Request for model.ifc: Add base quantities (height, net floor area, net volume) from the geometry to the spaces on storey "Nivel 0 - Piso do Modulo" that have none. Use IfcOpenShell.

First a look at what the model holds.

```python
import ifcopenshell
import ifcopenshell.util.element
import ifcopenshell.util.unit

model = ifcopenshell.open("model.ifc")
print(model.schema)
for unit_type in ("LENGTHUNIT", "AREAUNIT", "VOLUMEUNIT"):
    print(unit_type, ifcopenshell.util.unit.calculate_unit_scale(model, unit_type))
storey = next(s for s in model.by_type("IfcBuildingStorey") if s.Name == "Nivel 0 - Piso do Modulo")
spaces = [e for e in ifcopenshell.util.element.get_decomposition(storey) if e.is_a("IfcSpace")]
for e in sorted(spaces, key=lambda e: e.id()):
    print(e.id(), e.is_a(), e.Name, list(ifcopenshell.util.element.get_psets(e, qtos_only=True)), sep=" | ")
```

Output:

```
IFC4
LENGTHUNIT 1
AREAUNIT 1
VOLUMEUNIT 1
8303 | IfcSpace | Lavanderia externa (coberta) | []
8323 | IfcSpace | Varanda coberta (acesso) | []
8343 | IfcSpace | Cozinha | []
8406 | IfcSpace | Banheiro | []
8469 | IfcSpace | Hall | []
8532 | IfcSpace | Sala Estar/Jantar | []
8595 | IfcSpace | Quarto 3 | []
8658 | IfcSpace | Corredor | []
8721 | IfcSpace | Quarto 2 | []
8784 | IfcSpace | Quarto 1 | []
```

```python
import ifcopenshell
import ifcopenshell.api.pset
import ifcopenshell.geom
import ifcopenshell.util.element
import ifcopenshell.util.shape
import ifcopenshell.util.unit

model = ifcopenshell.open("model.ifc")
unit_scale = ifcopenshell.util.unit.calculate_unit_scale(model)
area_scale = ifcopenshell.util.unit.calculate_unit_scale(model, "AREAUNIT")
volume_scale = ifcopenshell.util.unit.calculate_unit_scale(model, "VOLUMEUNIT")
settings = ifcopenshell.geom.settings()

storey = next(s for s in model.by_type("IfcBuildingStorey") if s.Name == "Nivel 0 - Piso do Modulo")
spaces = [e for e in ifcopenshell.util.element.get_decomposition(storey) if e.is_a("IfcSpace")]

for e in sorted(spaces, key=lambda e: e.id()):
    if ifcopenshell.util.element.get_psets(e, qtos_only=True, should_inherit=False):
        continue
    # Geometry comes back in metres, in the element's own axes.
    shape = ifcopenshell.geom.create_shape(settings, e)
    values = {
        "Height": ifcopenshell.util.shape.get_z(shape.geometry) / unit_scale,
        "NetFloorArea": ifcopenshell.util.shape.get_footprint_area(shape.geometry) / area_scale,
        "NetVolume": ifcopenshell.util.shape.get_volume(shape.geometry) / volume_scale,
    }
    qto = ifcopenshell.api.pset.add_qto(model, product=e, name="Qto_SpaceBaseQuantities")
    ifcopenshell.api.pset.edit_qto(model, qto=qto, properties=values)
    print(e.id(), {k: round(v, 3) for k, v in values.items()})

model.write("model_rev.ifc")
```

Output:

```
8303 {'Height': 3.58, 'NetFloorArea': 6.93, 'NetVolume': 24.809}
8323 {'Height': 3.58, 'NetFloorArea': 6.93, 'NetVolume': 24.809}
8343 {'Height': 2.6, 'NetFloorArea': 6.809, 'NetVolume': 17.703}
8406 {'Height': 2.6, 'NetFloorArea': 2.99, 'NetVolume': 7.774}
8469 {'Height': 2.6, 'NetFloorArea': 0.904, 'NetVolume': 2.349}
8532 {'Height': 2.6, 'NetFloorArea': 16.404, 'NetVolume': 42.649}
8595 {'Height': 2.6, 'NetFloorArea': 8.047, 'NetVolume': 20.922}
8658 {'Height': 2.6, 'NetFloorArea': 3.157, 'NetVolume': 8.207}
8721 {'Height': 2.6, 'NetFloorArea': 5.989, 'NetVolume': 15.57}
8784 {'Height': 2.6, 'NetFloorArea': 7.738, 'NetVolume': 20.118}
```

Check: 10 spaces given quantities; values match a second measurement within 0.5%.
